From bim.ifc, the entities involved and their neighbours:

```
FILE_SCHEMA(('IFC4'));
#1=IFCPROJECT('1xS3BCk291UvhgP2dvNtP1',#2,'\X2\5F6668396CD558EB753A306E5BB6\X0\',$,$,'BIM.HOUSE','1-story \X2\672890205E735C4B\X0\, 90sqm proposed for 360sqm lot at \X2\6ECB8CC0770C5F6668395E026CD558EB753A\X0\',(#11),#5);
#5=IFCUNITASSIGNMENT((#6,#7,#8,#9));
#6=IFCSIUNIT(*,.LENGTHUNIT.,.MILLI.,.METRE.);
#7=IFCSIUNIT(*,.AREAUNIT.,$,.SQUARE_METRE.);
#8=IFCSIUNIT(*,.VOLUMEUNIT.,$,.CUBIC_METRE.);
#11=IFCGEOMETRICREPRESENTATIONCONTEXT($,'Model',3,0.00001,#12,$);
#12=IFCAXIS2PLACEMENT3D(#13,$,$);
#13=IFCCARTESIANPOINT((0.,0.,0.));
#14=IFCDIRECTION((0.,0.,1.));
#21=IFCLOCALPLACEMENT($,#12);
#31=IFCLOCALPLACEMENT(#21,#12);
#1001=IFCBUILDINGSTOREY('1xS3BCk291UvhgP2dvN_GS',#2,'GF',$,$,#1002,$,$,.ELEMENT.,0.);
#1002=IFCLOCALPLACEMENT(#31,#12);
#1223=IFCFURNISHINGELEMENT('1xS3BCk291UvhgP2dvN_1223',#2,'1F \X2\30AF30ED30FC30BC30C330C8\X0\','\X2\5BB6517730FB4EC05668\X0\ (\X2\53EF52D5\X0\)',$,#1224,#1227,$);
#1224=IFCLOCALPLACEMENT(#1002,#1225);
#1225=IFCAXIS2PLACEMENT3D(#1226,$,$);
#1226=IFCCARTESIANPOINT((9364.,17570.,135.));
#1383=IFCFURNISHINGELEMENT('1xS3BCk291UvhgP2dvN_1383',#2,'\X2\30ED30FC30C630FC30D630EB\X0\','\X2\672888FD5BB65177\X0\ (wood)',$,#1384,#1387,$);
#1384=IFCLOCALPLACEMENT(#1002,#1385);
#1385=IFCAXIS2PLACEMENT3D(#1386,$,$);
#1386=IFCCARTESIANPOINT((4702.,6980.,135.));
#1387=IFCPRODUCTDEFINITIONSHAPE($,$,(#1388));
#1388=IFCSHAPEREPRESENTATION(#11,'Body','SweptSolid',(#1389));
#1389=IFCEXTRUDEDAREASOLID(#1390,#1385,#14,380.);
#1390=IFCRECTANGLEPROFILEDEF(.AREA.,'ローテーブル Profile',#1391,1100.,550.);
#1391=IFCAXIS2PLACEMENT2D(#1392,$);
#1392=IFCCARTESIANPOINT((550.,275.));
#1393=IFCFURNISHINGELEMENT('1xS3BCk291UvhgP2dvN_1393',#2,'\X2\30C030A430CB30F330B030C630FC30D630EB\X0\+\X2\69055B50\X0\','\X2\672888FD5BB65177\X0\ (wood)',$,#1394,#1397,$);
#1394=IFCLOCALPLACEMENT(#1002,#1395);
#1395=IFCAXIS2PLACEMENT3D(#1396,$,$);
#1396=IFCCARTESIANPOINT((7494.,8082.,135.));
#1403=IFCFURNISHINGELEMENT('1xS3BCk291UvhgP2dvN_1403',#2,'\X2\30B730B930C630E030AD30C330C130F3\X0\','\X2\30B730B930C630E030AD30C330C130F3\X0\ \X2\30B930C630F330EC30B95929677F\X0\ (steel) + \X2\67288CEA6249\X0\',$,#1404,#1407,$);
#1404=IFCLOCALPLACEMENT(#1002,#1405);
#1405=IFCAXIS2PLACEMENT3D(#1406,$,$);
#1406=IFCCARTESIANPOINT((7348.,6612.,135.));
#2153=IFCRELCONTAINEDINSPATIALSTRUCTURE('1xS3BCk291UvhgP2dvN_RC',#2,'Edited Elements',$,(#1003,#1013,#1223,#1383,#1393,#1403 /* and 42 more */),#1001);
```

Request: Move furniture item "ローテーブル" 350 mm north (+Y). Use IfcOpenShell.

```python
import ifcopenshell
import ifcopenshell.api.geometry
import ifcopenshell.util.placement
import ifcopenshell.util.unit

model = ifcopenshell.open("bim.ifc")
unit_scale = ifcopenshell.util.unit.calculate_unit_scale(model)

item = model.by_guid("1xS3BCk291UvhgP2dvN_1383")
matrix = ifcopenshell.util.placement.get_local_placement(item.ObjectPlacement)
matrix[1, 3] += 0.35 / unit_scale
ifcopenshell.api.geometry.edit_object_placement(model, product=item, matrix=matrix, is_si=False)

print(ifcopenshell.util.placement.get_local_placement(item.ObjectPlacement).round(3) + 0.0)

model.write("bim_updated.ifc")
```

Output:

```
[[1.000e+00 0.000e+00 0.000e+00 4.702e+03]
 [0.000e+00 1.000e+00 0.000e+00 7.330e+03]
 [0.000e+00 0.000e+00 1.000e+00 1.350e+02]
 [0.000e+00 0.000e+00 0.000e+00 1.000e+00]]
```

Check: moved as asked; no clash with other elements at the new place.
